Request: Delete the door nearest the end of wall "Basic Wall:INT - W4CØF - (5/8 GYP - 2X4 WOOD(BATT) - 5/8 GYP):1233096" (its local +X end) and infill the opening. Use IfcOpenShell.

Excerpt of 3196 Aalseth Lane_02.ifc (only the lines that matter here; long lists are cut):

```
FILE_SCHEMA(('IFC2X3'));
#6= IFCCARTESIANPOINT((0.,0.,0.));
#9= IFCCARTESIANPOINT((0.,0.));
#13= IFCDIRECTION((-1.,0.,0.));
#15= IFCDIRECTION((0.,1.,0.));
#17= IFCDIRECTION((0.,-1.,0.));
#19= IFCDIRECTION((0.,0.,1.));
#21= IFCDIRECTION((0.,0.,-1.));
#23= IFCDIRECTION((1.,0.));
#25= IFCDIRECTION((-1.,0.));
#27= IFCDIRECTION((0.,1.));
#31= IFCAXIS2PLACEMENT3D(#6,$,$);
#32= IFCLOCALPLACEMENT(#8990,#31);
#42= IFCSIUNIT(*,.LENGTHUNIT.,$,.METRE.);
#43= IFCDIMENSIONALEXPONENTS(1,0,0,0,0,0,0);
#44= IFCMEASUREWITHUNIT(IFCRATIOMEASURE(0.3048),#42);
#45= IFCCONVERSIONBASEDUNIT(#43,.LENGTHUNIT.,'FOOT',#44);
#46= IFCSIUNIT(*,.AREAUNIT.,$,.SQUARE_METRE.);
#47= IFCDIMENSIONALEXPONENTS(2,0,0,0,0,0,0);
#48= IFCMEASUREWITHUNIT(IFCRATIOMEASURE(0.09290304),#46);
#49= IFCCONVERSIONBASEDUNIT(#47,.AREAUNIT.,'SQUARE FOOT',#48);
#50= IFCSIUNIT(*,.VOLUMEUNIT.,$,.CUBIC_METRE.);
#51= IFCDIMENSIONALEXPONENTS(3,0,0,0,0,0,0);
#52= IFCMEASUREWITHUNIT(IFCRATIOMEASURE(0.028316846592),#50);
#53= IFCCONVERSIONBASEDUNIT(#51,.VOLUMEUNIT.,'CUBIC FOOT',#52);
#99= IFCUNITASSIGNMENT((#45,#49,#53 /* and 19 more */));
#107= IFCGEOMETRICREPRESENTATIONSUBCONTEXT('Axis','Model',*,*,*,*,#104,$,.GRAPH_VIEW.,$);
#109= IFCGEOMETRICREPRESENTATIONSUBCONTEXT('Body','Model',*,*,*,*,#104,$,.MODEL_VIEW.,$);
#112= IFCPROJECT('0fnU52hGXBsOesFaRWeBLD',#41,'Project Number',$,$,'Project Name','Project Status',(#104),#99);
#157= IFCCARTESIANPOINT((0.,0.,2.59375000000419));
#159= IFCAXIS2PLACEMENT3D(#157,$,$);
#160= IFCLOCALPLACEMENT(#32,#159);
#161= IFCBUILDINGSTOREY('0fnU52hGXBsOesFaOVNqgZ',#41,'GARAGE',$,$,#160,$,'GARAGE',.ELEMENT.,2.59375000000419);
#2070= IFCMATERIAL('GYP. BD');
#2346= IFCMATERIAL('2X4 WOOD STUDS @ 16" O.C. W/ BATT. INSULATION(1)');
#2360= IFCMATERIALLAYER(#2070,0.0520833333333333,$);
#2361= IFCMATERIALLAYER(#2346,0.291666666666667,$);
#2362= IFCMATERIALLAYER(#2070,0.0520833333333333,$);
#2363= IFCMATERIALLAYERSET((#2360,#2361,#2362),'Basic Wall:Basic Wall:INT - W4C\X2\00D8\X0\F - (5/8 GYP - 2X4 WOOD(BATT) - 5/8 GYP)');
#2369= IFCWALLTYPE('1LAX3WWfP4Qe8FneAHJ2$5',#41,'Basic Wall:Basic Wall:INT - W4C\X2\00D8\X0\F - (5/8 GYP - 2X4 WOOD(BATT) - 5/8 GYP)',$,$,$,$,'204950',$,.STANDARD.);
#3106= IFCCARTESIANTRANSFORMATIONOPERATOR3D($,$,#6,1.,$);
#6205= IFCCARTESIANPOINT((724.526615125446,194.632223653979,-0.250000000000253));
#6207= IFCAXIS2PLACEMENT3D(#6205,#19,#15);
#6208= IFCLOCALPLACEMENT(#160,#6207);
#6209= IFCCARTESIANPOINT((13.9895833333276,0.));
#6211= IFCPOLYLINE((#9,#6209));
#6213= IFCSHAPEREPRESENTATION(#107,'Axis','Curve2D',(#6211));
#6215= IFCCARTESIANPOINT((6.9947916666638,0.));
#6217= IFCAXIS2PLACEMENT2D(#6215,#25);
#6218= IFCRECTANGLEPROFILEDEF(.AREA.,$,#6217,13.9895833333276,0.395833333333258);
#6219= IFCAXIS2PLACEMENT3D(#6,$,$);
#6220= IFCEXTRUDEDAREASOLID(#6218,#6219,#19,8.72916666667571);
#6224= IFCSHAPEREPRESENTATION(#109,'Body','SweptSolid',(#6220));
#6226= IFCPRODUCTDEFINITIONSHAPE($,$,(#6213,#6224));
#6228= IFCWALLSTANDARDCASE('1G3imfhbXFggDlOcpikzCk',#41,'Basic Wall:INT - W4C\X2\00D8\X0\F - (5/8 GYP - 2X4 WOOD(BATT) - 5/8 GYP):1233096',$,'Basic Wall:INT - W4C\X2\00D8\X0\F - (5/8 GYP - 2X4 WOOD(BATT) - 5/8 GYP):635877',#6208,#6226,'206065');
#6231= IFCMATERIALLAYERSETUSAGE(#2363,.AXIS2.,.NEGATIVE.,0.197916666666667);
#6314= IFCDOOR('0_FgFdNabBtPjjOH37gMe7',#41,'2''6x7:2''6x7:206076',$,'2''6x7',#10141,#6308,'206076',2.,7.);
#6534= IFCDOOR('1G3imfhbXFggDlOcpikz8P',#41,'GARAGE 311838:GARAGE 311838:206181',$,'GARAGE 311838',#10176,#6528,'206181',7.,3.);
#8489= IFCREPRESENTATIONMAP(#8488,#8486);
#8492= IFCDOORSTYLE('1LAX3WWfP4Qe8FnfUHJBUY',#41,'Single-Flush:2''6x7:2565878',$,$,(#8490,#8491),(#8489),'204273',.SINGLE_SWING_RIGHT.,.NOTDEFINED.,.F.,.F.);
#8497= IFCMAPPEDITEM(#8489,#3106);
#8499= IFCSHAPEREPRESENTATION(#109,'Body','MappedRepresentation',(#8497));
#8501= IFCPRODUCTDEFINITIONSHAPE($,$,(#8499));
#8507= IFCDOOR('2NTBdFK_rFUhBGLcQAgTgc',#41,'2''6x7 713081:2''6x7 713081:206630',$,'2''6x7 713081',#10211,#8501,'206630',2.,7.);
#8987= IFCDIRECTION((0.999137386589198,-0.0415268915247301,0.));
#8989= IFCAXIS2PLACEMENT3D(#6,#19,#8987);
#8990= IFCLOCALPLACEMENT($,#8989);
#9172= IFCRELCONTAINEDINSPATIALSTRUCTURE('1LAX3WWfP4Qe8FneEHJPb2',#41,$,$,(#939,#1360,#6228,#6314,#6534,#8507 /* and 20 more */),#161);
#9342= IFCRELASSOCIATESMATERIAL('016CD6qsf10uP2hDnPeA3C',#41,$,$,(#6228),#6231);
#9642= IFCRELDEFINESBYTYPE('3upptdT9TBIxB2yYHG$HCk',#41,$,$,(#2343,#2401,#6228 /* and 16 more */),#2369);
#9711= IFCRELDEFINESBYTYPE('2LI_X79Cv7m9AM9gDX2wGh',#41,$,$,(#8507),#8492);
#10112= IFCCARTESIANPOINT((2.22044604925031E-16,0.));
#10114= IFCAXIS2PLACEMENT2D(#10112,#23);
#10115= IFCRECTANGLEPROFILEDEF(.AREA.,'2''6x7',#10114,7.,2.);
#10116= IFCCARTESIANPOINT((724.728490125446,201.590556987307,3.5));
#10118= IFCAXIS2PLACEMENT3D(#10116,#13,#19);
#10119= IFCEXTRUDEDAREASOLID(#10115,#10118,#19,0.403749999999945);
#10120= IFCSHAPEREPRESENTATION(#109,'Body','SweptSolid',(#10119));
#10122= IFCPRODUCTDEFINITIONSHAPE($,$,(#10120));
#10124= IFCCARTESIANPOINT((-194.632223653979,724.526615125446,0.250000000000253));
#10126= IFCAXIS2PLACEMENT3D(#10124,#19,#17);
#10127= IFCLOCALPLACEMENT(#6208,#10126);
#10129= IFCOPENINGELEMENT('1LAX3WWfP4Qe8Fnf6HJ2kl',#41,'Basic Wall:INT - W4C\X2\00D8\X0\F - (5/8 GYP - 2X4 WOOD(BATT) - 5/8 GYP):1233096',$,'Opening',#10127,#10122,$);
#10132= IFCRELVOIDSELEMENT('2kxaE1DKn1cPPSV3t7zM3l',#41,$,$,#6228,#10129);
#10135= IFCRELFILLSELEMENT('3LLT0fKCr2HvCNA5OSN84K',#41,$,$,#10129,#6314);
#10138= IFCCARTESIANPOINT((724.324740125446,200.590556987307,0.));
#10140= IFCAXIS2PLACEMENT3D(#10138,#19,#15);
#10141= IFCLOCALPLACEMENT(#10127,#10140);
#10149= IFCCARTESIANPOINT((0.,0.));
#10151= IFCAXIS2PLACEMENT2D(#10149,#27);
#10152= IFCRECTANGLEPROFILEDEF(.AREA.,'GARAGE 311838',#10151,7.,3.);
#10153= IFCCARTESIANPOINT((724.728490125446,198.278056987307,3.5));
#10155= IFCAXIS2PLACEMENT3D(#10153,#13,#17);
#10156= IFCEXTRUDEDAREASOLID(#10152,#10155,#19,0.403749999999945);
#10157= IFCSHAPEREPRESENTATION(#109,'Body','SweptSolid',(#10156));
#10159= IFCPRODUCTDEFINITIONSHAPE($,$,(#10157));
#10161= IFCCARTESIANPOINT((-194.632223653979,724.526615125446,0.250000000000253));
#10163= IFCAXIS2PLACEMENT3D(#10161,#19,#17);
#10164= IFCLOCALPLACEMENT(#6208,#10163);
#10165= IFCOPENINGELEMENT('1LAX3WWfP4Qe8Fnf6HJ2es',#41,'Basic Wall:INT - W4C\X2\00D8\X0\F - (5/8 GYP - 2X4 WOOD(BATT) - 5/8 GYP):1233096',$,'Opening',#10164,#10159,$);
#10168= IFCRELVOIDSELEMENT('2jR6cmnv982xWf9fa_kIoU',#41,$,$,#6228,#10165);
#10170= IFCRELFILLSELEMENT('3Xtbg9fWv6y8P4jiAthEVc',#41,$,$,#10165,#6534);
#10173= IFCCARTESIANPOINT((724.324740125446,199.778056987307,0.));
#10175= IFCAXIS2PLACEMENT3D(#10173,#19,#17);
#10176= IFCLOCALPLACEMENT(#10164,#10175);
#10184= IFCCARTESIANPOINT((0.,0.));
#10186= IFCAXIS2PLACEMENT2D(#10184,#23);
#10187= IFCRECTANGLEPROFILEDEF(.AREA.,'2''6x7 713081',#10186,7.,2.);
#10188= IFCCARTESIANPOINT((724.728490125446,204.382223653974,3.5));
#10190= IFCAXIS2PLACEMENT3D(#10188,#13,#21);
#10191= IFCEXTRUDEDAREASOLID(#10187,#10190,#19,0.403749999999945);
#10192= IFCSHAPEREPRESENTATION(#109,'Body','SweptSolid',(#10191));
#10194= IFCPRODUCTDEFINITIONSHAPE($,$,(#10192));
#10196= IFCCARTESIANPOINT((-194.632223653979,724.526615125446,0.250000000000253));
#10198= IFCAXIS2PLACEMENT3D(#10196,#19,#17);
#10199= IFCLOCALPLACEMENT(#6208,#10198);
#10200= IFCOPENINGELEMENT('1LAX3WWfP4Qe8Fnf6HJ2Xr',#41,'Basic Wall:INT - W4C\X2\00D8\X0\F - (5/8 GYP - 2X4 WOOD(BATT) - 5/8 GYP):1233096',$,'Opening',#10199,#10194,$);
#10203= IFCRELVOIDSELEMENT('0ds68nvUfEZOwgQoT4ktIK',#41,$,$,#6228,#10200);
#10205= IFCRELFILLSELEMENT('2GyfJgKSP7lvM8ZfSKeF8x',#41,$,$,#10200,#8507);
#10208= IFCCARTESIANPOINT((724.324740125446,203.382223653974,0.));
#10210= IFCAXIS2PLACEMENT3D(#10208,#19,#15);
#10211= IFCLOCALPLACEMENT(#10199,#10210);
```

```python
import ifcopenshell
import ifcopenshell.api.feature
import ifcopenshell.api.root
import ifcopenshell.geom
import ifcopenshell.util.shape

model = ifcopenshell.open("3196 Aalseth Lane_02.ifc")
settings = ifcopenshell.geom.settings()


def volume(element):
    """Net volume in cubic metres, openings subtracted."""
    shape = ifcopenshell.geom.create_shape(settings, element)
    return ifcopenshell.util.shape.get_volume(shape.geometry)


door = model.by_guid("2NTBdFK_rFUhBGLcQAgTgc")
opening = door.FillsVoids[0].RelatingOpeningElement
wall = opening.VoidsElements[0].RelatingBuildingElement
before = volume(wall)

ifcopenshell.api.root.remove_product(model, product=door)
ifcopenshell.api.feature.remove_feature(model, feature=opening)

after = volume(wall)

print(f"wall volume {before:.3f} -> {after:.3f} m3")

model.write("3196 Aalseth Lane_02_updated.ifc")
```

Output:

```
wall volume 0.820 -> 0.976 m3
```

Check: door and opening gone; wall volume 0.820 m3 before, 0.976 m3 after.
